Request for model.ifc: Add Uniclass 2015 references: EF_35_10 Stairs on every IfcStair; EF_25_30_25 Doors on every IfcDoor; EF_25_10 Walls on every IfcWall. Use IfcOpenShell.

First a look at what the model holds.

```python
import ifcopenshell

model = ifcopenshell.open("model.ifc")
print(model.schema)
print("classifications:", [c.Name for c in model.by_type("IfcClassification")])
for ifc_class in ("IfcDoor", "IfcRoof", "IfcStair", "IfcWall", "IfcWindow"):
    print(ifc_class, len(model.by_type(ifc_class)))
```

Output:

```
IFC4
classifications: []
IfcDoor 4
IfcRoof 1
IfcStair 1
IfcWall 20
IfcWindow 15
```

```python
import ifcopenshell
import ifcopenshell.api.classification

model = ifcopenshell.open("model.ifc")

system = ifcopenshell.api.classification.add_classification(model, classification="Uniclass 2015")

codes = {
    "IfcStair": ("EF_35_10", "Stairs"),
    "IfcDoor": ("EF_25_30_25", "Doors"),
    "IfcWall": ("EF_25_10", "Walls"),
}
for ifc_class, (code, name) in codes.items():
    products = model.by_type(ifc_class)
    ifcopenshell.api.classification.add_reference(
        model, products=products, classification=system, identification=code, name=name
    )
    print(code, len(products))

model.write("model_v2.ifc")
```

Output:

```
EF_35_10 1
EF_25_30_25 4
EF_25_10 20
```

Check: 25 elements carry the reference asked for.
